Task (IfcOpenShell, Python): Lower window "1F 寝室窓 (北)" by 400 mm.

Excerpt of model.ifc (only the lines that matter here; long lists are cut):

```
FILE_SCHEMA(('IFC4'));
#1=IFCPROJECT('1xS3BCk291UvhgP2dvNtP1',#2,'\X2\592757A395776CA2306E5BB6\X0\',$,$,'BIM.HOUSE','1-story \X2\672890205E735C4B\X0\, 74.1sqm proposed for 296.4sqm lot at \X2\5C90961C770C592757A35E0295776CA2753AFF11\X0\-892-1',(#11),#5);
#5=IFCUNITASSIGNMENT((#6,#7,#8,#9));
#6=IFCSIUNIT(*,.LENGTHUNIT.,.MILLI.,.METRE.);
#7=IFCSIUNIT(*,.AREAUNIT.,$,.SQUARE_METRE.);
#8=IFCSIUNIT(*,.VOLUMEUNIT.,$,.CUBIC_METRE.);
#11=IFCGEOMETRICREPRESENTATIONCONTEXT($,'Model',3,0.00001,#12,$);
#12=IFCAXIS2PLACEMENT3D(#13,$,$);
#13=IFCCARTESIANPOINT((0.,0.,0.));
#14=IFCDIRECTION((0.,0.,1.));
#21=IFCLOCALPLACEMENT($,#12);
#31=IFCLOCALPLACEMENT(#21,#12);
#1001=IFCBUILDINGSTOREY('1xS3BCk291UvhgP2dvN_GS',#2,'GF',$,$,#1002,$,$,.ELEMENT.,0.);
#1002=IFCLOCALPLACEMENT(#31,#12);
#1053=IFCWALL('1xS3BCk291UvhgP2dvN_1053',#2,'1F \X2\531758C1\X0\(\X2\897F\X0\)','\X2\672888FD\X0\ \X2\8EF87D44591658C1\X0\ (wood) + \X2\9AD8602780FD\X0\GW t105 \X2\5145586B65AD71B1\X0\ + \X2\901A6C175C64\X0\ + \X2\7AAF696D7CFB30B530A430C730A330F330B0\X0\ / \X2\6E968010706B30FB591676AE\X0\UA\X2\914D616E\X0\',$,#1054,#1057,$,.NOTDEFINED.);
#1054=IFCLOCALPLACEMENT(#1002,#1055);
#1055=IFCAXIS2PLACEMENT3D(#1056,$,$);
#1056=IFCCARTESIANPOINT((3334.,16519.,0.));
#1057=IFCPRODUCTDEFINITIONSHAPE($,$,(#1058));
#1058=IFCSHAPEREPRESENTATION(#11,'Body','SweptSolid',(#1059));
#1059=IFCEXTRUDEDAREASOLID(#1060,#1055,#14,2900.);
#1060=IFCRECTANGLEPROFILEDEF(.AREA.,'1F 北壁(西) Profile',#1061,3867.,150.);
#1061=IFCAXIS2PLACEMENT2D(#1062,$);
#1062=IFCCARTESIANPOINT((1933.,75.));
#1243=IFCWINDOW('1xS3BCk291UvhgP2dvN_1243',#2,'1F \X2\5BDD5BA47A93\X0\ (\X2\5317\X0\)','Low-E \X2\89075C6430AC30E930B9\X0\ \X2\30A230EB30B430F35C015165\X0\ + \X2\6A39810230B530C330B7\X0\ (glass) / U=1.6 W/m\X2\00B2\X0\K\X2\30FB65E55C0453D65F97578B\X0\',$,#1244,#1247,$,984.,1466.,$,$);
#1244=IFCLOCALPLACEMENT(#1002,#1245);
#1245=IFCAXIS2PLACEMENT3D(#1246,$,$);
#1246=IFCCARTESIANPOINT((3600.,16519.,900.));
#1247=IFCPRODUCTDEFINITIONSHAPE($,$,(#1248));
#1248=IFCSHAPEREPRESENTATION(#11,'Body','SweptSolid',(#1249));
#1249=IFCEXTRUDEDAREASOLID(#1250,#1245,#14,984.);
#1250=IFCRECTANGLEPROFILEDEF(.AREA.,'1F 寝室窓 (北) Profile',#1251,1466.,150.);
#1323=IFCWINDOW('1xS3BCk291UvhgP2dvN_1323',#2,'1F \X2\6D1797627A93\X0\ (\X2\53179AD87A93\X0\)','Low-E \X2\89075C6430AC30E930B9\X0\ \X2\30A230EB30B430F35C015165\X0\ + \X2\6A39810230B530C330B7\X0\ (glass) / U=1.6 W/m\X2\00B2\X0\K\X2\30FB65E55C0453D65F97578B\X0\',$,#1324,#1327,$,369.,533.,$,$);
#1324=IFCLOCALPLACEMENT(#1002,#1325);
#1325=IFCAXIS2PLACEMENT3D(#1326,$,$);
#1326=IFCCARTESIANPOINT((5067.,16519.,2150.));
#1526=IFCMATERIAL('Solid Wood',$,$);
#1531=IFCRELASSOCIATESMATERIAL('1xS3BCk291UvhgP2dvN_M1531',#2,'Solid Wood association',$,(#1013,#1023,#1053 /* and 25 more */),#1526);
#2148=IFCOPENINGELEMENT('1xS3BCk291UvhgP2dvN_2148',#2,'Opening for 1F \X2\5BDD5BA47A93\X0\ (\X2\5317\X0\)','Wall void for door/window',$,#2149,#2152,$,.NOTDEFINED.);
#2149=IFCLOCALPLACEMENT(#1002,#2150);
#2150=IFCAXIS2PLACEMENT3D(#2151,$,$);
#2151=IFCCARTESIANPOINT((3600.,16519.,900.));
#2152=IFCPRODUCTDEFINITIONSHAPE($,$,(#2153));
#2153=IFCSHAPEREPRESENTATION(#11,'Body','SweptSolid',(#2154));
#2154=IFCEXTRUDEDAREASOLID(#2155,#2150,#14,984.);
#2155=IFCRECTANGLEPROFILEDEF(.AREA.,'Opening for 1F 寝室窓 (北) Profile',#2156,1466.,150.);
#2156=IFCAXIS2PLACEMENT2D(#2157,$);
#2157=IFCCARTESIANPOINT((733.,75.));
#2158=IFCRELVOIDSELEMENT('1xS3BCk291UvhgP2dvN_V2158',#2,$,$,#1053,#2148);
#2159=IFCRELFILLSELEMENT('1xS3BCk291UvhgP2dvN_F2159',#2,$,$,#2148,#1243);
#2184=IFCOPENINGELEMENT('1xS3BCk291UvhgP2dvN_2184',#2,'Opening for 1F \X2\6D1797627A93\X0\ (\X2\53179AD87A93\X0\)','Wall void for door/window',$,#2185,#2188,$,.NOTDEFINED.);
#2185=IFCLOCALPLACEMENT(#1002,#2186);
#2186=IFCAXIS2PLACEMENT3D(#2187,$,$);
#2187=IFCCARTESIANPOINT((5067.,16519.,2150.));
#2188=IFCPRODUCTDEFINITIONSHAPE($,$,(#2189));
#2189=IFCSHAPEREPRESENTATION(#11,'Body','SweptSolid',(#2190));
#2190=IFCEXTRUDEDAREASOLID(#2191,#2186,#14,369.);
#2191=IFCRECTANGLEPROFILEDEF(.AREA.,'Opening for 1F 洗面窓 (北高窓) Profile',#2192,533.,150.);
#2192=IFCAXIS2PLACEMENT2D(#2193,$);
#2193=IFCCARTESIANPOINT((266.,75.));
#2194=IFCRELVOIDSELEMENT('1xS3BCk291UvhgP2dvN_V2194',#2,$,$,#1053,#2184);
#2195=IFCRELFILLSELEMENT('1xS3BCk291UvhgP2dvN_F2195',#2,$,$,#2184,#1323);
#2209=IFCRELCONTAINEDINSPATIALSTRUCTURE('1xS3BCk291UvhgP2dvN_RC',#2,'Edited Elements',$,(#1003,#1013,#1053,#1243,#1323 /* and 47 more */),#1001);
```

```python
import numpy as np
import ifcopenshell
import ifcopenshell.api.geometry
import ifcopenshell.util.placement
import ifcopenshell.util.unit

model = ifcopenshell.open("model.ifc")
unit_scale = ifcopenshell.util.unit.calculate_unit_scale(model)

window = model.by_id(1243)
opening = window.FillsVoids[0].RelatingOpeningElement
dz = -0.4 / unit_scale

shift = np.array([0.0, 0.0, dz])
# The window is not placed relative to its opening, so move both.
for product in (opening, window):
    matrix = ifcopenshell.util.placement.get_local_placement(product.ObjectPlacement)
    matrix[:3, 3] += shift
    ifcopenshell.api.geometry.edit_object_placement(model, product=product, matrix=matrix, is_si=False)

print(f"moved by {dz * unit_scale:+.3f} m")

model.write("model-out.ifc")
```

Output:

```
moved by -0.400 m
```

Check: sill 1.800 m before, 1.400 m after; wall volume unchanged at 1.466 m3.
